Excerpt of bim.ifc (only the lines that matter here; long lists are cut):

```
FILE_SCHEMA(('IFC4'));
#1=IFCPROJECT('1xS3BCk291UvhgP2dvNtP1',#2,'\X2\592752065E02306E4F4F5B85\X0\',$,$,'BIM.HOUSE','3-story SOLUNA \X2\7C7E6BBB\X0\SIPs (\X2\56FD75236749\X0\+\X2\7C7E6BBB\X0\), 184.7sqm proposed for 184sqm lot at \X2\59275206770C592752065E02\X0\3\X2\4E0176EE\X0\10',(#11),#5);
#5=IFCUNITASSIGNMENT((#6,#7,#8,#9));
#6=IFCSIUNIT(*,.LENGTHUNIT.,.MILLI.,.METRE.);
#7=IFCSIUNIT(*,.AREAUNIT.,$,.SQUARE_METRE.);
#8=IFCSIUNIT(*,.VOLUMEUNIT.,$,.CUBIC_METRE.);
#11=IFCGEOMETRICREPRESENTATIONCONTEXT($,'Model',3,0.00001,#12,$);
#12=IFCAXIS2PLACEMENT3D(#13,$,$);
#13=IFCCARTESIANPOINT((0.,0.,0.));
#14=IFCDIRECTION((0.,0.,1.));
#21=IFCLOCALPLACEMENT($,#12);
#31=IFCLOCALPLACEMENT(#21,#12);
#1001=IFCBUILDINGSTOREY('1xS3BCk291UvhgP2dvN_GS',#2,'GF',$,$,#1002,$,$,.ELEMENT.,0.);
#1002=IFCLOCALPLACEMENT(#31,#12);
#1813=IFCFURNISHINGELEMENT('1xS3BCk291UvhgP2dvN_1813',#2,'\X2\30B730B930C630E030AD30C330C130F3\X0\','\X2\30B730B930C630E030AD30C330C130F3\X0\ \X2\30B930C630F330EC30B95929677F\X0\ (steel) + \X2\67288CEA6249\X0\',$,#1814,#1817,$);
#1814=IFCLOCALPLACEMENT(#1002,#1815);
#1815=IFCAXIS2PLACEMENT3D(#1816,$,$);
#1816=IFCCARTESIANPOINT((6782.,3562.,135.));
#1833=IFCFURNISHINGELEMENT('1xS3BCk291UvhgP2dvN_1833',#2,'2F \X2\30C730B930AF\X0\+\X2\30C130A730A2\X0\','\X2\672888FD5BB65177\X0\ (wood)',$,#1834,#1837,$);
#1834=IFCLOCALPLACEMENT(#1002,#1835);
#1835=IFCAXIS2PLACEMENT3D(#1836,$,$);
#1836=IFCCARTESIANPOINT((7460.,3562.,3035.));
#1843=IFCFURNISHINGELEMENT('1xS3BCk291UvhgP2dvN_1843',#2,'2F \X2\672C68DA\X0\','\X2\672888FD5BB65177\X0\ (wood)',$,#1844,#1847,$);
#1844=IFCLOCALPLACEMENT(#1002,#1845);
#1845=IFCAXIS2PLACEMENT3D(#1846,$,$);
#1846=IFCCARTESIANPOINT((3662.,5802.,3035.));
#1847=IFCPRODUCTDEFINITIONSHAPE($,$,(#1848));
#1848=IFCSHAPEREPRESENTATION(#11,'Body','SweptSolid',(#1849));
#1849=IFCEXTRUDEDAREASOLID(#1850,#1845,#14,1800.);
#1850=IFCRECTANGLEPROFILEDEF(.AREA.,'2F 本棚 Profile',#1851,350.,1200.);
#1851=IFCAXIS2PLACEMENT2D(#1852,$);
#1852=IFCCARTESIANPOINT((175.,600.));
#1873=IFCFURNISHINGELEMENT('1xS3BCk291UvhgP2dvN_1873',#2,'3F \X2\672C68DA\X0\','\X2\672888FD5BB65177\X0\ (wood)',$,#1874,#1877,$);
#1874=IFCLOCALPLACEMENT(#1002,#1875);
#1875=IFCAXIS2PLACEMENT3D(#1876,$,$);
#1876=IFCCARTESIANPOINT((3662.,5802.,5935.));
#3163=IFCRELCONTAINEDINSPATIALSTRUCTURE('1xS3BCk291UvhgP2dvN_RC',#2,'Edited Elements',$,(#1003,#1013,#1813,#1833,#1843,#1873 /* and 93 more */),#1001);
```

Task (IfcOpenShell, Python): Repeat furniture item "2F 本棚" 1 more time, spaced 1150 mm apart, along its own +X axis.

```python
import ifcopenshell
import ifcopenshell.api.geometry
import ifcopenshell.api.root
import ifcopenshell.util.element
import ifcopenshell.util.placement
import ifcopenshell.util.unit

model = ifcopenshell.open("bim.ifc")
unit_scale = ifcopenshell.util.unit.calculate_unit_scale(model)


def reuse_history(source, copy):
    """copy_class also copies each property set's owner history, people and application; keep the originals."""
    for rel in copy.IsDefinedBy:
        if rel.is_a("IfcRelDefinesByProperties") and (history := rel.RelatingPropertyDefinition.OwnerHistory):
            rel.RelatingPropertyDefinition.OwnerHistory = source.OwnerHistory
            ifcopenshell.util.element.remove_deep2(model, history)


source = model.by_guid("1xS3BCk291UvhgP2dvN_1843")
base = ifcopenshell.util.placement.get_local_placement(source.ObjectPlacement)
step = base[:3, 0] * 1.15 / unit_scale

for i in range(1, 2):
    copy = ifcopenshell.api.root.copy_class(model, product=source)
    copy.Representation = ifcopenshell.util.element.copy_deep(
        model, source.Representation, exclude=["IfcGeometricRepresentationContext", "IfcRepresentationMap"]
    )
    reuse_history(source, copy)
    matrix = base.copy()
    matrix[:3, 3] += i * step
    print("added at", matrix[:3, 3].round(3) + 0.0)
    ifcopenshell.api.geometry.edit_object_placement(model, product=copy, matrix=matrix, is_si=False)

model.write("bim_edited.ifc")
```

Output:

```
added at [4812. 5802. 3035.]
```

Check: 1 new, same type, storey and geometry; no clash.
